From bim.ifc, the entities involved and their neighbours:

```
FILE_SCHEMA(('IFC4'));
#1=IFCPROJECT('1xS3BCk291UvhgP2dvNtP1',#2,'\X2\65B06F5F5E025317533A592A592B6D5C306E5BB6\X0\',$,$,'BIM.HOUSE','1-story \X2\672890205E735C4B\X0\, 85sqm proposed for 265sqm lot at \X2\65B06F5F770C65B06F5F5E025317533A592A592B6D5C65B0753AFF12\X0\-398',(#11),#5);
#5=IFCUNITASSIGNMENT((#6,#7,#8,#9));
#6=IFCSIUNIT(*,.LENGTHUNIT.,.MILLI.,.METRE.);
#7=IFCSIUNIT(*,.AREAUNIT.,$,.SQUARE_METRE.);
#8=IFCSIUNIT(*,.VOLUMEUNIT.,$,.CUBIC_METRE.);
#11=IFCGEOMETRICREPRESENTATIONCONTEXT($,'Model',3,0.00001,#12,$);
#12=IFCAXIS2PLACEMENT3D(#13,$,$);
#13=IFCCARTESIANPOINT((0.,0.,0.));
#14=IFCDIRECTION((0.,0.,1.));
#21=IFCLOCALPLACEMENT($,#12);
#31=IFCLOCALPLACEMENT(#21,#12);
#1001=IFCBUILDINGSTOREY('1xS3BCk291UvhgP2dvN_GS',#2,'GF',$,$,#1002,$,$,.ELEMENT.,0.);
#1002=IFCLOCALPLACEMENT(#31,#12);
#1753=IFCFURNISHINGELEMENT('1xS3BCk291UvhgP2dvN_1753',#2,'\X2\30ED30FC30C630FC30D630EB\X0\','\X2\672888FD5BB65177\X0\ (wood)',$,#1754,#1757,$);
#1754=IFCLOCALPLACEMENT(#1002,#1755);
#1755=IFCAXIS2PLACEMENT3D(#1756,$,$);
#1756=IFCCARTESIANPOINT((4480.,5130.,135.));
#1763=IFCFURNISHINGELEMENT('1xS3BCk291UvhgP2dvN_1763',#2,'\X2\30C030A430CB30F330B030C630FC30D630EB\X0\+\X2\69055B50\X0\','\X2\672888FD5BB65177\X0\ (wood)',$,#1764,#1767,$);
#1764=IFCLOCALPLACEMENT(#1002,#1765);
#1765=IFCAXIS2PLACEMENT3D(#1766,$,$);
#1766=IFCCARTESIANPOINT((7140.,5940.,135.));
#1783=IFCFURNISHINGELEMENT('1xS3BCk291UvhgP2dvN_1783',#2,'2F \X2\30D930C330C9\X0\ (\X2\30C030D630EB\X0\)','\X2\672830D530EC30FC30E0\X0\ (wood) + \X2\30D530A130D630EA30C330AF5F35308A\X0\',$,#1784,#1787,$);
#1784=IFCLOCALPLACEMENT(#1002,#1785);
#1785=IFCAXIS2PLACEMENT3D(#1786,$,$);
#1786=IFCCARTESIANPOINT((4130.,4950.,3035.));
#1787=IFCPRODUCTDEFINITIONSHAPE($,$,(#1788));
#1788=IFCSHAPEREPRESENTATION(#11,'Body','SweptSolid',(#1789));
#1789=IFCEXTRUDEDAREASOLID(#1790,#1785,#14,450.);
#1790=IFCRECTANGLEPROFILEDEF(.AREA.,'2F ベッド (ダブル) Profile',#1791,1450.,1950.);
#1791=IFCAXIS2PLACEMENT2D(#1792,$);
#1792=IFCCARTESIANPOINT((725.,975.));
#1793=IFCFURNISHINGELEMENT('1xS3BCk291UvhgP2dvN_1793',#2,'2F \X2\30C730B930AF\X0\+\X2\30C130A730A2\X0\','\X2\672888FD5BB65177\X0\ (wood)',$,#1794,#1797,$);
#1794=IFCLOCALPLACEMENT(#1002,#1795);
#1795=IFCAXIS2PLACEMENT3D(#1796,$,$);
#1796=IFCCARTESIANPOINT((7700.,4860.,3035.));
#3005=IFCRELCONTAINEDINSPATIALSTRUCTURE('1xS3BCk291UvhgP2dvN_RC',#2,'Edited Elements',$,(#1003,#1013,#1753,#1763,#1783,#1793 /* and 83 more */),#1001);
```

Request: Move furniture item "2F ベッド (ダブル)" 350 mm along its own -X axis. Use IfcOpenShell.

```python
import ifcopenshell
import ifcopenshell.api.geometry
import ifcopenshell.util.placement

model = ifcopenshell.open("bim.ifc")

item = model.by_guid("1xS3BCk291UvhgP2dvN_1783")
matrix = ifcopenshell.util.placement.get_local_placement(item.ObjectPlacement)
matrix[:3, 3] -= matrix[:3, 0] * 350.0
ifcopenshell.api.geometry.edit_object_placement(model, product=item, matrix=matrix, is_si=False)

print(ifcopenshell.util.placement.get_local_placement(item.ObjectPlacement).round(3) + 0.0)

model.write("bim_rev.ifc")
```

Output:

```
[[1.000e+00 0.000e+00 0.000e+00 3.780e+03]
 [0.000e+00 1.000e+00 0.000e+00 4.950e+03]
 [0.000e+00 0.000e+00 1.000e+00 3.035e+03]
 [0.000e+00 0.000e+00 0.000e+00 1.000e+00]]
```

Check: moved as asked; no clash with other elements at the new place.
